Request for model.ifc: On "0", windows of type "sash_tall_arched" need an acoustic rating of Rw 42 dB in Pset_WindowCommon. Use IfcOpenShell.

First a look at what the model holds.

```python
import ifcopenshell
import ifcopenshell.util.element

model = ifcopenshell.open("model.ifc")
print(model.schema)
storey = next(s for s in model.by_type("IfcBuildingStorey") if s.Name == "0")
windows = [e for e in ifcopenshell.util.element.get_decomposition(storey) if e.is_a("IfcWindow")]
seen = {}
for e in windows:
    element_type = ifcopenshell.util.element.get_type(e)
    key = (element_type.Name if element_type != e and element_type else None, ifcopenshell.util.element.get_pset(e, "Pset_WindowCommon", "AcousticRating"))
    seen[key] = seen.get(key, 0) + 1
for (name, value), count in sorted(seen.items(), key=str):
    print(count, "x", name, "|", value)
```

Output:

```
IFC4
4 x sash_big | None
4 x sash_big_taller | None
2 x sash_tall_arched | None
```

```python
import ifcopenshell
import ifcopenshell.api.pset
import ifcopenshell.util.element

model = ifcopenshell.open("model.ifc")

storey = next(s for s in model.by_type("IfcBuildingStorey") if s.Name == "0")
windows = [e for e in ifcopenshell.util.element.get_decomposition(storey) if e.is_a("IfcWindow")]

count = 0
for e in windows:
    element_type = ifcopenshell.util.element.get_type(e)
    if element_type in (None, e) or element_type.Name != "sash_tall_arched":
        continue
    # add_pset returns the element's existing set when there is one.
    pset = ifcopenshell.api.pset.add_pset(model, product=e, name="Pset_WindowCommon")
    ifcopenshell.api.pset.edit_pset(model, pset=pset, properties={"AcousticRating": "Rw 42 dB"})
    count += 1

print(count, "windows updated")

model.write("model_edited.ifc")
```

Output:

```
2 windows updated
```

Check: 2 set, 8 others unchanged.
